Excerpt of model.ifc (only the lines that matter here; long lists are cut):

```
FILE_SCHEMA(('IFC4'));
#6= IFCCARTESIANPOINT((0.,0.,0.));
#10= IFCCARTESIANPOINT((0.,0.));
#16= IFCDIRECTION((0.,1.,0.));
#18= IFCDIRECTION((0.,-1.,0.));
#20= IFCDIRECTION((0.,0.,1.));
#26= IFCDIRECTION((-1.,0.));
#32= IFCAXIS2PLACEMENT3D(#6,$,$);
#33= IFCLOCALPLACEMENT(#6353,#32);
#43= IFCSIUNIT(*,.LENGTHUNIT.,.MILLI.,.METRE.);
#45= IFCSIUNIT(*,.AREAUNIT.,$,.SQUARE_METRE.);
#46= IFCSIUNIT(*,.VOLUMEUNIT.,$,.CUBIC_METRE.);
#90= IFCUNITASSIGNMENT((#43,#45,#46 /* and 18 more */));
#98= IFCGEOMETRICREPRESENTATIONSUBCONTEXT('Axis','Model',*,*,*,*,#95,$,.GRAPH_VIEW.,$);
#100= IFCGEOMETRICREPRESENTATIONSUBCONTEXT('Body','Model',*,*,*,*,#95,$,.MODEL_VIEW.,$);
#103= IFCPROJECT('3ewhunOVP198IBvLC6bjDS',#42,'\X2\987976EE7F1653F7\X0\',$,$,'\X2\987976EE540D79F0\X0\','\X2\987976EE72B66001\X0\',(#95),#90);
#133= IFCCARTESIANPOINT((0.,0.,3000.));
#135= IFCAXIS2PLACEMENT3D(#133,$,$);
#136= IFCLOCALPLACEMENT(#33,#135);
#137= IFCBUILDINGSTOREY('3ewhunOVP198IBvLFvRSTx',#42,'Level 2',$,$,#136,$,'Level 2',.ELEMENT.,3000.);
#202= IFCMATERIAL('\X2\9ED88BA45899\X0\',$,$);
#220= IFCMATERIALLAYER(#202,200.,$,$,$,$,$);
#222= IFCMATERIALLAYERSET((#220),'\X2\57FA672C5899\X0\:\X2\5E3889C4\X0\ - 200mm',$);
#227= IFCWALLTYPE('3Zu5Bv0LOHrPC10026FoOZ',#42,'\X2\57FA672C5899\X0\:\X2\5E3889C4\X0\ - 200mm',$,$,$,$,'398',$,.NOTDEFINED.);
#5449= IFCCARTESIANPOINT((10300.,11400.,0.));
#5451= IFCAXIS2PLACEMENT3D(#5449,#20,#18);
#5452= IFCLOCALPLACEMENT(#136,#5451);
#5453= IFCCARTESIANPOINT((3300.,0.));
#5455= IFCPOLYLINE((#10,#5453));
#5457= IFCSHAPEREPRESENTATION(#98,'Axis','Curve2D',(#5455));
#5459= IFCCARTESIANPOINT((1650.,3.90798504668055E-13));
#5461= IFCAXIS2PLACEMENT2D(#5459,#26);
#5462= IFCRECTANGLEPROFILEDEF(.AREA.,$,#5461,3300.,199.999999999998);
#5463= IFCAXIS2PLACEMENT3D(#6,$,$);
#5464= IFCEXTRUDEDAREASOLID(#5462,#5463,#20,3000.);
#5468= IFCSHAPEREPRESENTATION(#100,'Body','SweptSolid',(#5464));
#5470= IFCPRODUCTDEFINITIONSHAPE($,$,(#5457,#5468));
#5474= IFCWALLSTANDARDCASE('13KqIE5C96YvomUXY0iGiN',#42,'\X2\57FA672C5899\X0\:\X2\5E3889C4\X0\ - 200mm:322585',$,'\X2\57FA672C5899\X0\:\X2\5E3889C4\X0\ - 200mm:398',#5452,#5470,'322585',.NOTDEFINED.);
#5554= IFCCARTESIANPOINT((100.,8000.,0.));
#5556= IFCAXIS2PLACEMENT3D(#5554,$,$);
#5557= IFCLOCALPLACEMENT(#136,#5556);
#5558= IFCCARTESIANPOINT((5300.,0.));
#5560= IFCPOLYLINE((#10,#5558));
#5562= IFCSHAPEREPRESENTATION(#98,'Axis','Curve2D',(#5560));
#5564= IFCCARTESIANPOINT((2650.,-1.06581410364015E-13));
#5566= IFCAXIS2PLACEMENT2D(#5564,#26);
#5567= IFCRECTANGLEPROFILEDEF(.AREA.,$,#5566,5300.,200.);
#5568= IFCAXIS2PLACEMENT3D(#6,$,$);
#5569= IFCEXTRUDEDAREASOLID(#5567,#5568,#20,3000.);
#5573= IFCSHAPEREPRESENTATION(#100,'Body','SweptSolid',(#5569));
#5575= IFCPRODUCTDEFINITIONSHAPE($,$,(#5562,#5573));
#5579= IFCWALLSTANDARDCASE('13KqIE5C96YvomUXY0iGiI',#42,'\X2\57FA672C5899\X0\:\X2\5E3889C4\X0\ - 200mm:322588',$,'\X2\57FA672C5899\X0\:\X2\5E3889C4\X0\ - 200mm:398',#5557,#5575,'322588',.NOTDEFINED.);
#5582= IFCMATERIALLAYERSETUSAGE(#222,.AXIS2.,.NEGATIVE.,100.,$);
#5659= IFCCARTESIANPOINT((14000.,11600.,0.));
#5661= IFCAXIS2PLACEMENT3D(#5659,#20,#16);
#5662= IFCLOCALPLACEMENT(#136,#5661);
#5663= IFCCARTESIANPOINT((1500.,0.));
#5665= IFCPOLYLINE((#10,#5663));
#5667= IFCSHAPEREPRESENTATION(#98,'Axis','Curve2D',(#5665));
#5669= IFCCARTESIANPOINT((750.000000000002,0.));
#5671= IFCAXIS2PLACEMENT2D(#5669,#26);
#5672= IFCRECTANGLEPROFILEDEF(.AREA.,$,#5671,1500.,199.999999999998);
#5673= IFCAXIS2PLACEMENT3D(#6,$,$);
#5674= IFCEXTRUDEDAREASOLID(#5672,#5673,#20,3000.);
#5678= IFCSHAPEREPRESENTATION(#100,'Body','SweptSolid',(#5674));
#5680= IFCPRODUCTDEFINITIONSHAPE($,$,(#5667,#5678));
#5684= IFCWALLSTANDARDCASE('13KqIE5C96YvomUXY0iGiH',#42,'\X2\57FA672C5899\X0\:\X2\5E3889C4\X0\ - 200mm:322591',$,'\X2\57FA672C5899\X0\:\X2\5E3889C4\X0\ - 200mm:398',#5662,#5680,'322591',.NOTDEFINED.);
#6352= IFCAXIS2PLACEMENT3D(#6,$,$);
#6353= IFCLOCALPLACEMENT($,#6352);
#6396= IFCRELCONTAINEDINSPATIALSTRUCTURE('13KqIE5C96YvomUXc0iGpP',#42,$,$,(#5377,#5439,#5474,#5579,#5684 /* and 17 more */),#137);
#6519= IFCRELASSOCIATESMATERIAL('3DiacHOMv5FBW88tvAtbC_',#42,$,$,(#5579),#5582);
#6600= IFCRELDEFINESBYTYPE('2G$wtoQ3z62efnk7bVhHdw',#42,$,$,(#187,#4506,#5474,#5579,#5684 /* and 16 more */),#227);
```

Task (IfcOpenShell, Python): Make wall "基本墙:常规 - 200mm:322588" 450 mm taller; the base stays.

```python
import ifcopenshell
import ifcopenshell.geom
import ifcopenshell.util.representation
import ifcopenshell.util.shape

model = ifcopenshell.open("model.ifc")
settings = ifcopenshell.geom.settings()


def volume(element):
    """Net volume in cubic metres, openings subtracted."""
    shape = ifcopenshell.geom.create_shape(settings, element)
    return ifcopenshell.util.shape.get_volume(shape.geometry)


wall = model.by_id(5579)
before = volume(wall)

body = ifcopenshell.util.representation.get_representation(wall, "Model", "Body")
solid = body.Items[0]
old_height = solid.Depth
solid.Depth += 450.0
after = volume(wall)

print(f"height {old_height:g} -> {solid.Depth:g}, volume {before:.3f} -> {after:.3f} m3")

model.write("model_rev.ifc")
```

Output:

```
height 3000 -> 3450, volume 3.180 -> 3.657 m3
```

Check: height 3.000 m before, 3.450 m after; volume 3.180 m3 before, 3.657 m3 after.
